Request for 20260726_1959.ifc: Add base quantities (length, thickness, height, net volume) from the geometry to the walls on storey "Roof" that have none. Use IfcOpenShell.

First a look at what the model holds.

```python
import ifcopenshell
import ifcopenshell.util.element
import ifcopenshell.util.unit

model = ifcopenshell.open("20260726_1959.ifc")
print(model.schema)
for unit_type in ("LENGTHUNIT", "AREAUNIT", "VOLUMEUNIT"):
    print(unit_type, ifcopenshell.util.unit.calculate_unit_scale(model, unit_type))
storey = next(s for s in model.by_type("IfcBuildingStorey") if s.Name == "Roof")
walls = [e for e in ifcopenshell.util.element.get_decomposition(storey) if e.is_a("IfcWall")]
for e in sorted(walls, key=lambda e: e.id()):
    print(e.id(), e.is_a(), e.Name, list(ifcopenshell.util.element.get_psets(e, qtos_only=True)), sep=" | ")
```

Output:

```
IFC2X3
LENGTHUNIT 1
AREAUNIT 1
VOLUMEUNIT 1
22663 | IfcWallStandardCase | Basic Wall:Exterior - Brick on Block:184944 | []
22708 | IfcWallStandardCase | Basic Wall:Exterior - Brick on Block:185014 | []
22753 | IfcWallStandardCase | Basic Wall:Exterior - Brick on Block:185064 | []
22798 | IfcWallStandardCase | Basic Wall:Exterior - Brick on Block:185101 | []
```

```python
import ifcopenshell
import ifcopenshell.api.pset
import ifcopenshell.geom
import ifcopenshell.util.element
import ifcopenshell.util.shape
import ifcopenshell.util.unit

model = ifcopenshell.open("20260726_1959.ifc")
unit_scale = ifcopenshell.util.unit.calculate_unit_scale(model)
volume_scale = ifcopenshell.util.unit.calculate_unit_scale(model, "VOLUMEUNIT")
settings = ifcopenshell.geom.settings()

storey = next(s for s in model.by_type("IfcBuildingStorey") if s.Name == "Roof")
walls = [e for e in ifcopenshell.util.element.get_decomposition(storey) if e.is_a("IfcWall")]

for e in sorted(walls, key=lambda e: e.id()):
    if ifcopenshell.util.element.get_psets(e, qtos_only=True, should_inherit=False):
        continue
    # Geometry comes back in metres, in the element's own axes.
    shape = ifcopenshell.geom.create_shape(settings, e)
    values = {
        "Length": ifcopenshell.util.shape.get_x(shape.geometry) / unit_scale,
        "Width": ifcopenshell.util.shape.get_y(shape.geometry) / unit_scale,
        "Height": ifcopenshell.util.shape.get_z(shape.geometry) / unit_scale,
        "NetVolume": ifcopenshell.util.shape.get_volume(shape.geometry) / volume_scale,
    }
    qto = ifcopenshell.api.pset.add_qto(model, product=e, name="BaseQuantities")
    ifcopenshell.api.pset.edit_qto(model, qto=qto, properties=values)
    print(e.id(), {k: round(v, 3) for k, v in values.items()})

model.write("20260726_1959_rev.ifc")
```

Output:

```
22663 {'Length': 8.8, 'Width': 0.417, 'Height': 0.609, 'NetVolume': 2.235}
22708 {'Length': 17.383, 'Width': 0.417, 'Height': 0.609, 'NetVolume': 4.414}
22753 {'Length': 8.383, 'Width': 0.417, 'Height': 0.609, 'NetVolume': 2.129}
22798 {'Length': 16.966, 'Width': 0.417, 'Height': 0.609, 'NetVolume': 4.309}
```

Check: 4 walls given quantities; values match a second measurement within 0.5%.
